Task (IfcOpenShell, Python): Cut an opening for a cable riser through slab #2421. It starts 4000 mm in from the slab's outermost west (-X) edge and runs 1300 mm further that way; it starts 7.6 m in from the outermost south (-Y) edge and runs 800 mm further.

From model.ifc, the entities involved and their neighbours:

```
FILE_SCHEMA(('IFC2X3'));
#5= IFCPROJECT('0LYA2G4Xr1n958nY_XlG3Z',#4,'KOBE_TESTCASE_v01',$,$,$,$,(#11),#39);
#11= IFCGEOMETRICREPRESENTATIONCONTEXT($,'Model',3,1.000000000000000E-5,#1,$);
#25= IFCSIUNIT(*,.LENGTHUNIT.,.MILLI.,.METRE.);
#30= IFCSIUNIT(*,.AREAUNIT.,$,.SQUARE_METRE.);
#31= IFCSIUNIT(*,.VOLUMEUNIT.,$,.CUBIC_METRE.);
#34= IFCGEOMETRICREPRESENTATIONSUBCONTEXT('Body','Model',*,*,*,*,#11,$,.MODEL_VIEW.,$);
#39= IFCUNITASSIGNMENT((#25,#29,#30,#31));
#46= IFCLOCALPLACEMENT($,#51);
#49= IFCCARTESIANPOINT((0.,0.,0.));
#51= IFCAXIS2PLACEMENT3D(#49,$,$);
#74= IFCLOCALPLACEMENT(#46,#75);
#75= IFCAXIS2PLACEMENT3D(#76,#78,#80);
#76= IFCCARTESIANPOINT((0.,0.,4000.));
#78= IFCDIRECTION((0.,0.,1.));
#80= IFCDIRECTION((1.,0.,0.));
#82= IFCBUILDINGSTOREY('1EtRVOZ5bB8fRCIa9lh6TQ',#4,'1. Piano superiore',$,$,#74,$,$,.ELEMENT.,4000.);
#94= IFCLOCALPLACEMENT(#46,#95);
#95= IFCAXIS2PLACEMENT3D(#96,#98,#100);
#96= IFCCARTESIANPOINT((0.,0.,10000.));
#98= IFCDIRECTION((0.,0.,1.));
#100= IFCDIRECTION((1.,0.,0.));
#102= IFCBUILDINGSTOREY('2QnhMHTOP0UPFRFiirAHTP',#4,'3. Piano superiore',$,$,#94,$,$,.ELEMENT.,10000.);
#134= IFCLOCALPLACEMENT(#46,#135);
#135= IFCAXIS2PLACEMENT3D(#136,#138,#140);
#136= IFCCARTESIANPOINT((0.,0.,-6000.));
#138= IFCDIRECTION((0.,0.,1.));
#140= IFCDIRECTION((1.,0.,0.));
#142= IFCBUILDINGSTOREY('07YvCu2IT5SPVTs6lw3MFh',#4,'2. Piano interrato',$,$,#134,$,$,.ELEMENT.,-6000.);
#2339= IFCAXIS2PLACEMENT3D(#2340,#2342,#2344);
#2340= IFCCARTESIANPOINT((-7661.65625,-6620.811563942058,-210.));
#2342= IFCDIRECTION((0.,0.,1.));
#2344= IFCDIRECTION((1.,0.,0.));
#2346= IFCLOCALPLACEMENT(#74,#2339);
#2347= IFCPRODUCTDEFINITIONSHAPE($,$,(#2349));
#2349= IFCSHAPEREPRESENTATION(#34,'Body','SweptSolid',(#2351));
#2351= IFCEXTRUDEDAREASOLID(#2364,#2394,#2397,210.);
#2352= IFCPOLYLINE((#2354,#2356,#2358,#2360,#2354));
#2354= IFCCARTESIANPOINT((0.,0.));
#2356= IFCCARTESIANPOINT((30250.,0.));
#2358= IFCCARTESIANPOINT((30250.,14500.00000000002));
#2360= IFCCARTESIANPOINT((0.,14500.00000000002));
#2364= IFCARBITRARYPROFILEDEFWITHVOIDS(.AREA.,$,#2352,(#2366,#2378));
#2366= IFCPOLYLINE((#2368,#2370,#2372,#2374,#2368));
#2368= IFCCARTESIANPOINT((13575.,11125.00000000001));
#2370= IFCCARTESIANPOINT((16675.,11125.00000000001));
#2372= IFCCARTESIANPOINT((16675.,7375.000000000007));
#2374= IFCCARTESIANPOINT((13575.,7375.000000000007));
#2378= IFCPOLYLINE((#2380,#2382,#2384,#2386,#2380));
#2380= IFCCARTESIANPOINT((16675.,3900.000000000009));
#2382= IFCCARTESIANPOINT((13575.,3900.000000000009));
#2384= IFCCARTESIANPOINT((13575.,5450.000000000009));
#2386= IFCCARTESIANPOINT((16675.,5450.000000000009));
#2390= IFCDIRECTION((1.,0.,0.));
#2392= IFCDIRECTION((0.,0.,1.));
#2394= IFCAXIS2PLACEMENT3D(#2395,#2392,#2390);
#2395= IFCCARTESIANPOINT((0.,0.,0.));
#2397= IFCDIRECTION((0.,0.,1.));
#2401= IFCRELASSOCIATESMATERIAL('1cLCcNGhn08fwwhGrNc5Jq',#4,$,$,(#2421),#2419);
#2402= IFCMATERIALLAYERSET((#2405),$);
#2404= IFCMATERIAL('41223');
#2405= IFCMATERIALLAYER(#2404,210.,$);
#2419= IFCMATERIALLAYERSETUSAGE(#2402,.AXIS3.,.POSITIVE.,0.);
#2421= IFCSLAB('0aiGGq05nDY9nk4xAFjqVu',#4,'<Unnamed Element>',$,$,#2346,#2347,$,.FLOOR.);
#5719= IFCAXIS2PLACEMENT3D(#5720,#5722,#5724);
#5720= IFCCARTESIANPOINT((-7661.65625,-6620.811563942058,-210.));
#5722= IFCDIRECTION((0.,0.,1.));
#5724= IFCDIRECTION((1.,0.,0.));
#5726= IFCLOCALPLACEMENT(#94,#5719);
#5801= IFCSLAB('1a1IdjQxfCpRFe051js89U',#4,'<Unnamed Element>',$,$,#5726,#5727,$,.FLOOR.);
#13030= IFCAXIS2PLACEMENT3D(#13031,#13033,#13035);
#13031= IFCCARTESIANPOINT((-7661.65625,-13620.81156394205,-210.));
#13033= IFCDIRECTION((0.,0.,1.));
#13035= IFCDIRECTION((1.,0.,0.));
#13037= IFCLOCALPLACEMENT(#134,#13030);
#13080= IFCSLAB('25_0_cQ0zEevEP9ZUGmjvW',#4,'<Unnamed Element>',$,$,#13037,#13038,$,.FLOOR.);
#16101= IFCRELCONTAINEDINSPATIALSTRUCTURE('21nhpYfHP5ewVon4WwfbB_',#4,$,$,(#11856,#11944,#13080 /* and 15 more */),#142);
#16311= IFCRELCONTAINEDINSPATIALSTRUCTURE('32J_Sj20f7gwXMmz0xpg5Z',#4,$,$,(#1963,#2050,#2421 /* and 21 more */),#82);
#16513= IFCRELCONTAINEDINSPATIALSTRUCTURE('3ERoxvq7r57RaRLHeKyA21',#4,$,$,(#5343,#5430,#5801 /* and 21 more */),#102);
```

```python
import numpy as np
import ifcopenshell
import ifcopenshell.api.feature
import ifcopenshell.api.geometry
import ifcopenshell.api.root
import ifcopenshell.geom
import ifcopenshell.util.placement
import ifcopenshell.util.representation
import ifcopenshell.util.shape
import ifcopenshell.util.unit

model = ifcopenshell.open("model.ifc")
unit_scale = ifcopenshell.util.unit.calculate_unit_scale(model)
settings = ifcopenshell.geom.settings()


def volume(element):
    """Net volume in cubic metres, openings subtracted."""
    shape = ifcopenshell.geom.create_shape(settings, element)
    return ifcopenshell.util.shape.get_volume(shape.geometry)


slab = model.by_id(2421)
before = volume(slab)

# Extent in the slab's own axes, in metres. The edges named are its -X and -Y sides.
slab_shape = ifcopenshell.geom.create_shape(settings, slab)
vertices = ifcopenshell.util.shape.get_vertices(slab_shape.geometry)
x_min, y_min, bottom = vertices.min(axis=0)
top = vertices[:, 2].max()

opening = ifcopenshell.api.root.create_entity(model, ifc_class="IfcOpeningElement", name="Cable riser opening")
context = ifcopenshell.util.representation.get_context(model, "Model", "Body", "MODEL_VIEW")
width, depth = 1.3, 0.8
outline = [(0.0, 0.0), (width, 0.0), (width, depth), (0.0, depth), (0.0, 0.0)]
# Overshoot both faces by 50 mm so the cut is clean.
shape = ifcopenshell.api.geometry.add_slab_representation(
    model, context=context, depth=top - bottom + 0.1, polyline=outline
)
ifcopenshell.api.geometry.assign_representation(model, product=opening, representation=shape)

matrix = ifcopenshell.util.placement.get_local_placement(slab.ObjectPlacement)
matrix[:, 3] = matrix @ np.append(np.array([x_min + 4, y_min + 7.6, bottom - 0.05]) / unit_scale, 1.0)
ifcopenshell.api.geometry.edit_object_placement(model, product=opening, matrix=matrix, is_si=False)
ifcopenshell.api.feature.add_feature(model, feature=opening, element=slab)

after = volume(slab)

print(f"slab volume {before:.3f} -> {after:.3f} m3")

model.write("model-out.ifc")
```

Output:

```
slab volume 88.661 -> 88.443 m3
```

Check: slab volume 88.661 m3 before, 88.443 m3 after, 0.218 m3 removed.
